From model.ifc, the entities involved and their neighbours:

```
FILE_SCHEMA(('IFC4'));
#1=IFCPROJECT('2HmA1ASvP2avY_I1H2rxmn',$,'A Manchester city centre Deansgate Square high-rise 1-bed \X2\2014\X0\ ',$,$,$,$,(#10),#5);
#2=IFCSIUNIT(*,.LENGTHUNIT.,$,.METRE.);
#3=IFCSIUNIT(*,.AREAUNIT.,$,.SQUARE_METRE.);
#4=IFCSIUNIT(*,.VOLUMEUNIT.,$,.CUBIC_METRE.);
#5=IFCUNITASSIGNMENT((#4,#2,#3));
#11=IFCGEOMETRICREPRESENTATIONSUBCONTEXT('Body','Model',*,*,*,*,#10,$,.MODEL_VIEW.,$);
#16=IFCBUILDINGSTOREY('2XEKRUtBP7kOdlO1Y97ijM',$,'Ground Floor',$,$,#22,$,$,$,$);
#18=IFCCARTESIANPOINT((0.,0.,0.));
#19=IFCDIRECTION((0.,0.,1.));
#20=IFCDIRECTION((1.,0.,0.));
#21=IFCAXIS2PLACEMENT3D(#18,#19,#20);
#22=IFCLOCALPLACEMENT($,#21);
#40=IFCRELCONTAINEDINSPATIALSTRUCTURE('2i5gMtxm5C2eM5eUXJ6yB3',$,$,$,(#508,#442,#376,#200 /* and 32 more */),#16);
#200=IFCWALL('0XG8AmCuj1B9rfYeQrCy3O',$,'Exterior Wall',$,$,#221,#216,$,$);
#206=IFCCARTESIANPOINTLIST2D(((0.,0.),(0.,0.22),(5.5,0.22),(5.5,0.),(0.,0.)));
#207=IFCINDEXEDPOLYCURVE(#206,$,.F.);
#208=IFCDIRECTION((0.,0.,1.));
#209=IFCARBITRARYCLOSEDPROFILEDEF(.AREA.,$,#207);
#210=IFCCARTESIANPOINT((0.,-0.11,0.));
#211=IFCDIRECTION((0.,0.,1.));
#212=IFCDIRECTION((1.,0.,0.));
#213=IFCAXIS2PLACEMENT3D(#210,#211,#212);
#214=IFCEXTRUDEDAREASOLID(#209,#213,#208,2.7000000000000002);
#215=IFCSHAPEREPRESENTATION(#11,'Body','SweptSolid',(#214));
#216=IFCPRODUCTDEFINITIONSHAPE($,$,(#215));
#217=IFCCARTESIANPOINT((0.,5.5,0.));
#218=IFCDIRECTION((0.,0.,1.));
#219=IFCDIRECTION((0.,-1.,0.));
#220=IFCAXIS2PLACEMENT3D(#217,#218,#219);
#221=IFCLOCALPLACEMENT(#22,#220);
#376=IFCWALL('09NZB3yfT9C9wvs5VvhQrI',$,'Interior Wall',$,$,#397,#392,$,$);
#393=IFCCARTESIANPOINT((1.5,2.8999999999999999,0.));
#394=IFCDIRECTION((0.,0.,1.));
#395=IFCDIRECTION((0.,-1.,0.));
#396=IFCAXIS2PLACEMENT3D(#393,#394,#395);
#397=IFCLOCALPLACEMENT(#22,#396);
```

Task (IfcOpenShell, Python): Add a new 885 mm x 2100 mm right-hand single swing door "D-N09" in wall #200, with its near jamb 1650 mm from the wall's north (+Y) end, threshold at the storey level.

```python
import numpy as np
import ifcopenshell
import ifcopenshell.api.feature
import ifcopenshell.api.geometry
import ifcopenshell.api.root
import ifcopenshell.api.spatial
import ifcopenshell.geom
import ifcopenshell.util.element
import ifcopenshell.util.placement
import ifcopenshell.util.representation
import ifcopenshell.util.shape
import ifcopenshell.util.unit

model = ifcopenshell.open("model.ifc")
unit_scale = ifcopenshell.util.unit.calculate_unit_scale(model)
settings = ifcopenshell.geom.settings()


def volume(element):
    """Net volume in cubic metres, openings subtracted."""
    shape = ifcopenshell.geom.create_shape(settings, element)
    return ifcopenshell.util.shape.get_volume(shape.geometry)


wall = model.by_guid("0XG8AmCuj1B9rfYeQrCy3O")
storey = ifcopenshell.util.element.get_container(wall, ifc_class="IfcBuildingStorey")
context = ifcopenshell.util.representation.get_context(model, "Model", "Body", "MODEL_VIEW")
before = volume(wall)

width, height, from_end, sill = 0.885, 2.1, 1.65, 0.0  # metres

# The wall runs along its own X axis, and the end named is its -X end.
wall_shape = ifcopenshell.geom.create_shape(settings, wall)
x, y, z = ifcopenshell.util.shape.get_vertices(wall_shape.geometry).T
start = x.min() + from_end
face, thickness = float(y.min()), float(y.max() - y.min())
wall_matrix = ifcopenshell.util.placement.get_local_placement(wall.ObjectPlacement)
level = ifcopenshell.util.placement.get_local_placement(storey.ObjectPlacement)[2, 3]


def in_wall(x, y):
    """Placement at x, y metres in the wall's axes, at sill height."""
    matrix = wall_matrix.copy()
    matrix[:, 3] = wall_matrix @ np.array([x / unit_scale, y / unit_scale, 0.0, 1.0])
    matrix[2, 3] = level + sill / unit_scale
    return matrix


# Opening: a box that overshoots both wall faces by 50 mm.
opening = ifcopenshell.api.root.create_entity(model, ifc_class="IfcOpeningElement", predefined_type="OPENING")
box = ifcopenshell.api.geometry.add_wall_representation(
    model, context=context, length=width, height=height, thickness=thickness + 0.1
)
ifcopenshell.api.geometry.assign_representation(model, product=opening, representation=box)
ifcopenshell.api.geometry.edit_object_placement(model, product=opening, matrix=in_wall(start, face - 0.05), is_si=False)
ifcopenshell.api.feature.add_feature(model, feature=opening, element=wall)

door = ifcopenshell.api.root.create_entity(model, ifc_class="IfcDoor", name="D-N09", predefined_type="DOOR")
door.OverallWidth, door.OverallHeight = width / unit_scale, height / unit_scale
door.OperationType = "SINGLE_SWING_RIGHT"
body = ifcopenshell.api.geometry.add_door_representation(
    model,
    context=context,
    overall_width=door.OverallWidth,
    overall_height=door.OverallHeight,
    operation_type="SINGLE_SWING_RIGHT",
    lining_properties={"LiningDepth": thickness / unit_scale, "ThresholdDepth": thickness / unit_scale},
)
ifcopenshell.api.geometry.assign_representation(model, product=door, representation=body)
ifcopenshell.api.spatial.assign_container(model, products=[door], relating_structure=storey)
ifcopenshell.api.feature.add_filling(model, opening=opening, element=door)

# The lining spans the wall, so the door starts at the wall face.
ifcopenshell.api.geometry.edit_object_placement(model, product=door, matrix=in_wall(start, face), is_si=False)

after = volume(wall)

print(f"wall volume {before:.3f} -> {after:.3f} m3")

model.write("model_v2.ifc")
```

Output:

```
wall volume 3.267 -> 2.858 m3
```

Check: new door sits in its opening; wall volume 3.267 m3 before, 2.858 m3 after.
